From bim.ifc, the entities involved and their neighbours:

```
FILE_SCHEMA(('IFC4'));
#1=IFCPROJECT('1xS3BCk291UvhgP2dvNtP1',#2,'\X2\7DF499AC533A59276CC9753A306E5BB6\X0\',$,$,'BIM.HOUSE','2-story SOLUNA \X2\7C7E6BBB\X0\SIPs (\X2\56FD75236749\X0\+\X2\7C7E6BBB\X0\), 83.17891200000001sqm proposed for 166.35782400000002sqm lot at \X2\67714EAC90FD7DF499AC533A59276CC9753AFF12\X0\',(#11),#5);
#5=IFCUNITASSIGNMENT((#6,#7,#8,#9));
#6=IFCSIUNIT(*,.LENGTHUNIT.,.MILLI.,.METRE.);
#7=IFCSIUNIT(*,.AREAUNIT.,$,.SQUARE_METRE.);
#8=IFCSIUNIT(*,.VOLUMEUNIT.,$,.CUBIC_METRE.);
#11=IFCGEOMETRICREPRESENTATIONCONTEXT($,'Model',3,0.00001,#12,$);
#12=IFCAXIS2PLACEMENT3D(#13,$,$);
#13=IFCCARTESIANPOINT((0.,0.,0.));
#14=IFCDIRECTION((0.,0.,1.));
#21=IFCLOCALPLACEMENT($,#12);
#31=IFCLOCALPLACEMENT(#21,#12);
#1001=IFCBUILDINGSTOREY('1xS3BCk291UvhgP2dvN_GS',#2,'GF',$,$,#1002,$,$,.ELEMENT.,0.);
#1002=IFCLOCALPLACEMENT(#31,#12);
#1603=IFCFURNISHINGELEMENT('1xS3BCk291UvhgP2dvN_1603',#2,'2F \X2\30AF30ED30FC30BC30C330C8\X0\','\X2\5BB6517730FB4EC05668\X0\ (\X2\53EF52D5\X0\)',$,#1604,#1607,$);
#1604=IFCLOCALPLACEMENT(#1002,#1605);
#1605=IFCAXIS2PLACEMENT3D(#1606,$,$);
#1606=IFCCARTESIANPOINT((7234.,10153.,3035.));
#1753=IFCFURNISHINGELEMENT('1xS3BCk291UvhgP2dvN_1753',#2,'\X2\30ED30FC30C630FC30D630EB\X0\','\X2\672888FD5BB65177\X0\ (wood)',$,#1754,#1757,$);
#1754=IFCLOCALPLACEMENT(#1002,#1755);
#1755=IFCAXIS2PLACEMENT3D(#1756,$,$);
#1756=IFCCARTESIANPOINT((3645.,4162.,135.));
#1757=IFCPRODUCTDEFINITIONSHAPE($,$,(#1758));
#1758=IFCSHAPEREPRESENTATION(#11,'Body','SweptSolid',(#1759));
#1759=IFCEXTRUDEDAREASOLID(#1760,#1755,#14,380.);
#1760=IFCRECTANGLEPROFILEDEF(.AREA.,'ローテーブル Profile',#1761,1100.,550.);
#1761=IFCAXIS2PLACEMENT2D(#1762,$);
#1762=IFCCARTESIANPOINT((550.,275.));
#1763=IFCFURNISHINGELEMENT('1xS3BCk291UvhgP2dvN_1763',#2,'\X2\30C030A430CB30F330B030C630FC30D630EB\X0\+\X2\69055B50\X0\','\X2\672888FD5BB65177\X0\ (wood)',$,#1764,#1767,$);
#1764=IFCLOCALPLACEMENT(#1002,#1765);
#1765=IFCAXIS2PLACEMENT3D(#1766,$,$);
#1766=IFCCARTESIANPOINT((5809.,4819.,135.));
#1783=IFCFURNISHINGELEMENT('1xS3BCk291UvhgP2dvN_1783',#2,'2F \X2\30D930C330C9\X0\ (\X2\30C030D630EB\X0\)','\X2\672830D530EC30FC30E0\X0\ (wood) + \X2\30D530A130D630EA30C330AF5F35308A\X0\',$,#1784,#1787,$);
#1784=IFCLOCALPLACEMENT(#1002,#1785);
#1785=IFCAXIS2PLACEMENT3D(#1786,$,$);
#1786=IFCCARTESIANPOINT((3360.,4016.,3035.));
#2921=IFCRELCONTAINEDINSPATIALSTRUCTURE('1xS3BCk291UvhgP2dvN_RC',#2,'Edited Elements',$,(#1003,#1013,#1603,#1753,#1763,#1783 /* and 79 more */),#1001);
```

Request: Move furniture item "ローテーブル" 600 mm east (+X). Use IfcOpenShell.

```python
import ifcopenshell
import ifcopenshell.api.geometry
import ifcopenshell.util.placement

model = ifcopenshell.open("bim.ifc")

item = model.by_guid("1xS3BCk291UvhgP2dvN_1753")
matrix = ifcopenshell.util.placement.get_local_placement(item.ObjectPlacement)
matrix[0, 3] += 600.0
ifcopenshell.api.geometry.edit_object_placement(model, product=item, matrix=matrix, is_si=False)

print(ifcopenshell.util.placement.get_local_placement(item.ObjectPlacement).round(3) + 0.0)

model.write("bim_rev.ifc")
```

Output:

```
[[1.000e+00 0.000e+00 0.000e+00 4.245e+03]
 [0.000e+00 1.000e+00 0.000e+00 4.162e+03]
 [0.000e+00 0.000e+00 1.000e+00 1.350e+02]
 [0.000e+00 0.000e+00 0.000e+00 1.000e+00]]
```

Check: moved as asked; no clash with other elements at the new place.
